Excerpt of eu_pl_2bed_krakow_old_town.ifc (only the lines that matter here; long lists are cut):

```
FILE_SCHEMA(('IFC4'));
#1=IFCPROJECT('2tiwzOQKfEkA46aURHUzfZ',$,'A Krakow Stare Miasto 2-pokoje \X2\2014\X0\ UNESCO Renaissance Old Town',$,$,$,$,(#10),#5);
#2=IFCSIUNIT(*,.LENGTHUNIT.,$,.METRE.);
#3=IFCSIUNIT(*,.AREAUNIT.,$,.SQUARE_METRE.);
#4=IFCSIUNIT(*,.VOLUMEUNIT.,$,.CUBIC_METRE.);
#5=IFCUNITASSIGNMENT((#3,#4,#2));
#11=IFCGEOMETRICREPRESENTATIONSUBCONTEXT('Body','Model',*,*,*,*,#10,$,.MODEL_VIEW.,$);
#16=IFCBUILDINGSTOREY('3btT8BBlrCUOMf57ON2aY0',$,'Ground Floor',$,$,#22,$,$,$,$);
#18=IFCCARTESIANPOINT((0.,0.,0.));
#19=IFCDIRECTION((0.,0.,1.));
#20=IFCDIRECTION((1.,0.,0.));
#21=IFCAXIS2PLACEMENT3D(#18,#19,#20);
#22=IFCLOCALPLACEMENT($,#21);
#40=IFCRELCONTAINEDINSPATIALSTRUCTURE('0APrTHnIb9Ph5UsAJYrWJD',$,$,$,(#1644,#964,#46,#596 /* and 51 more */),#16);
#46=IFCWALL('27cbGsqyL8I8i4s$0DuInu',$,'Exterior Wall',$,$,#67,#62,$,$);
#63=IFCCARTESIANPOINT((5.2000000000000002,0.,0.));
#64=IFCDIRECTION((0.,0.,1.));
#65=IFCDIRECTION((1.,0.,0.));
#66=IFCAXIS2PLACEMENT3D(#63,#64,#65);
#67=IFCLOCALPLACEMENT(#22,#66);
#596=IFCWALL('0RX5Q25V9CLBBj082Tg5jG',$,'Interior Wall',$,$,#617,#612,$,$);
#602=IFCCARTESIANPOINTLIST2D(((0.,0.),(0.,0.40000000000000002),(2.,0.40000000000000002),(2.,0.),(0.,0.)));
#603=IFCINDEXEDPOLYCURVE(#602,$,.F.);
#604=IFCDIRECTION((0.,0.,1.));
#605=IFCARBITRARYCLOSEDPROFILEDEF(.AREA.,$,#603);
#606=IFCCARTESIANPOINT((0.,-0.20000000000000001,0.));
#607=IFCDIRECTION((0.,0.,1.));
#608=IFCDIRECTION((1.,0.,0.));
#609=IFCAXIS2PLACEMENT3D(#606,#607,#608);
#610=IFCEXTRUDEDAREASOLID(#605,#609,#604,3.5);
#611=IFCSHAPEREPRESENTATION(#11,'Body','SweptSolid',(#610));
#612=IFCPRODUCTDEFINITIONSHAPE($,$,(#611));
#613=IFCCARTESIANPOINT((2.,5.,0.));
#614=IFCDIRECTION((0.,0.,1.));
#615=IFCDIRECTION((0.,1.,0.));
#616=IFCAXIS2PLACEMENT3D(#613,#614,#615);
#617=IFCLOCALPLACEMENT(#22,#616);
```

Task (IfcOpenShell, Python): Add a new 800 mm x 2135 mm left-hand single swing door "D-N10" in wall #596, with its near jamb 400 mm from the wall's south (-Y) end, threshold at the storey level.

```python
import numpy as np
import ifcopenshell
import ifcopenshell.api.feature
import ifcopenshell.api.geometry
import ifcopenshell.api.root
import ifcopenshell.api.spatial
import ifcopenshell.geom
import ifcopenshell.util.element
import ifcopenshell.util.placement
import ifcopenshell.util.representation
import ifcopenshell.util.shape
import ifcopenshell.util.unit

model = ifcopenshell.open("eu_pl_2bed_krakow_old_town.ifc")
unit_scale = ifcopenshell.util.unit.calculate_unit_scale(model)
settings = ifcopenshell.geom.settings()


def volume(element):
    """Net volume in cubic metres, openings subtracted."""
    shape = ifcopenshell.geom.create_shape(settings, element)
    return ifcopenshell.util.shape.get_volume(shape.geometry)


wall = model.by_guid("0RX5Q25V9CLBBj082Tg5jG")
storey = ifcopenshell.util.element.get_container(wall, ifc_class="IfcBuildingStorey")
context = ifcopenshell.util.representation.get_context(model, "Model", "Body", "MODEL_VIEW")
before = volume(wall)

width, height, from_end, sill = 0.8, 2.135, 0.4, 0.0  # metres

# The wall runs along its own X axis, and the end named is its -X end.
wall_shape = ifcopenshell.geom.create_shape(settings, wall)
x, y, z = ifcopenshell.util.shape.get_vertices(wall_shape.geometry).T
start = x.min() + from_end
face, thickness = float(y.min()), float(y.max() - y.min())
wall_matrix = ifcopenshell.util.placement.get_local_placement(wall.ObjectPlacement)
level = ifcopenshell.util.placement.get_local_placement(storey.ObjectPlacement)[2, 3]


def in_wall(x, y):
    """Placement at x, y metres in the wall's axes, at sill height."""
    matrix = wall_matrix.copy()
    matrix[:, 3] = wall_matrix @ np.array([x / unit_scale, y / unit_scale, 0.0, 1.0])
    matrix[2, 3] = level + sill / unit_scale
    return matrix


# Opening: a box that overshoots both wall faces by 50 mm.
opening = ifcopenshell.api.root.create_entity(model, ifc_class="IfcOpeningElement", predefined_type="OPENING")
box = ifcopenshell.api.geometry.add_wall_representation(
    model, context=context, length=width, height=height, thickness=thickness + 0.1
)
ifcopenshell.api.geometry.assign_representation(model, product=opening, representation=box)
ifcopenshell.api.geometry.edit_object_placement(model, product=opening, matrix=in_wall(start, face - 0.05), is_si=False)
ifcopenshell.api.feature.add_feature(model, feature=opening, element=wall)

door = ifcopenshell.api.root.create_entity(model, ifc_class="IfcDoor", name="D-N10", predefined_type="DOOR")
door.OverallWidth, door.OverallHeight = width / unit_scale, height / unit_scale
door.OperationType = "SINGLE_SWING_LEFT"
body = ifcopenshell.api.geometry.add_door_representation(
    model,
    context=context,
    overall_width=door.OverallWidth,
    overall_height=door.OverallHeight,
    operation_type="SINGLE_SWING_LEFT",
    lining_properties={"LiningDepth": thickness / unit_scale, "ThresholdDepth": thickness / unit_scale},
)
ifcopenshell.api.geometry.assign_representation(model, product=door, representation=body)
ifcopenshell.api.spatial.assign_container(model, products=[door], relating_structure=storey)
ifcopenshell.api.feature.add_filling(model, opening=opening, element=door)

# The lining spans the wall, so the door starts at the wall face.
ifcopenshell.api.geometry.edit_object_placement(model, product=door, matrix=in_wall(start, face), is_si=False)

after = volume(wall)

print(f"wall volume {before:.3f} -> {after:.3f} m3")

model.write("eu_pl_2bed_krakow_old_town_rev.ifc")
```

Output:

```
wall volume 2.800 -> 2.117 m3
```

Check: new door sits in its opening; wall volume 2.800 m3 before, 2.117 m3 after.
